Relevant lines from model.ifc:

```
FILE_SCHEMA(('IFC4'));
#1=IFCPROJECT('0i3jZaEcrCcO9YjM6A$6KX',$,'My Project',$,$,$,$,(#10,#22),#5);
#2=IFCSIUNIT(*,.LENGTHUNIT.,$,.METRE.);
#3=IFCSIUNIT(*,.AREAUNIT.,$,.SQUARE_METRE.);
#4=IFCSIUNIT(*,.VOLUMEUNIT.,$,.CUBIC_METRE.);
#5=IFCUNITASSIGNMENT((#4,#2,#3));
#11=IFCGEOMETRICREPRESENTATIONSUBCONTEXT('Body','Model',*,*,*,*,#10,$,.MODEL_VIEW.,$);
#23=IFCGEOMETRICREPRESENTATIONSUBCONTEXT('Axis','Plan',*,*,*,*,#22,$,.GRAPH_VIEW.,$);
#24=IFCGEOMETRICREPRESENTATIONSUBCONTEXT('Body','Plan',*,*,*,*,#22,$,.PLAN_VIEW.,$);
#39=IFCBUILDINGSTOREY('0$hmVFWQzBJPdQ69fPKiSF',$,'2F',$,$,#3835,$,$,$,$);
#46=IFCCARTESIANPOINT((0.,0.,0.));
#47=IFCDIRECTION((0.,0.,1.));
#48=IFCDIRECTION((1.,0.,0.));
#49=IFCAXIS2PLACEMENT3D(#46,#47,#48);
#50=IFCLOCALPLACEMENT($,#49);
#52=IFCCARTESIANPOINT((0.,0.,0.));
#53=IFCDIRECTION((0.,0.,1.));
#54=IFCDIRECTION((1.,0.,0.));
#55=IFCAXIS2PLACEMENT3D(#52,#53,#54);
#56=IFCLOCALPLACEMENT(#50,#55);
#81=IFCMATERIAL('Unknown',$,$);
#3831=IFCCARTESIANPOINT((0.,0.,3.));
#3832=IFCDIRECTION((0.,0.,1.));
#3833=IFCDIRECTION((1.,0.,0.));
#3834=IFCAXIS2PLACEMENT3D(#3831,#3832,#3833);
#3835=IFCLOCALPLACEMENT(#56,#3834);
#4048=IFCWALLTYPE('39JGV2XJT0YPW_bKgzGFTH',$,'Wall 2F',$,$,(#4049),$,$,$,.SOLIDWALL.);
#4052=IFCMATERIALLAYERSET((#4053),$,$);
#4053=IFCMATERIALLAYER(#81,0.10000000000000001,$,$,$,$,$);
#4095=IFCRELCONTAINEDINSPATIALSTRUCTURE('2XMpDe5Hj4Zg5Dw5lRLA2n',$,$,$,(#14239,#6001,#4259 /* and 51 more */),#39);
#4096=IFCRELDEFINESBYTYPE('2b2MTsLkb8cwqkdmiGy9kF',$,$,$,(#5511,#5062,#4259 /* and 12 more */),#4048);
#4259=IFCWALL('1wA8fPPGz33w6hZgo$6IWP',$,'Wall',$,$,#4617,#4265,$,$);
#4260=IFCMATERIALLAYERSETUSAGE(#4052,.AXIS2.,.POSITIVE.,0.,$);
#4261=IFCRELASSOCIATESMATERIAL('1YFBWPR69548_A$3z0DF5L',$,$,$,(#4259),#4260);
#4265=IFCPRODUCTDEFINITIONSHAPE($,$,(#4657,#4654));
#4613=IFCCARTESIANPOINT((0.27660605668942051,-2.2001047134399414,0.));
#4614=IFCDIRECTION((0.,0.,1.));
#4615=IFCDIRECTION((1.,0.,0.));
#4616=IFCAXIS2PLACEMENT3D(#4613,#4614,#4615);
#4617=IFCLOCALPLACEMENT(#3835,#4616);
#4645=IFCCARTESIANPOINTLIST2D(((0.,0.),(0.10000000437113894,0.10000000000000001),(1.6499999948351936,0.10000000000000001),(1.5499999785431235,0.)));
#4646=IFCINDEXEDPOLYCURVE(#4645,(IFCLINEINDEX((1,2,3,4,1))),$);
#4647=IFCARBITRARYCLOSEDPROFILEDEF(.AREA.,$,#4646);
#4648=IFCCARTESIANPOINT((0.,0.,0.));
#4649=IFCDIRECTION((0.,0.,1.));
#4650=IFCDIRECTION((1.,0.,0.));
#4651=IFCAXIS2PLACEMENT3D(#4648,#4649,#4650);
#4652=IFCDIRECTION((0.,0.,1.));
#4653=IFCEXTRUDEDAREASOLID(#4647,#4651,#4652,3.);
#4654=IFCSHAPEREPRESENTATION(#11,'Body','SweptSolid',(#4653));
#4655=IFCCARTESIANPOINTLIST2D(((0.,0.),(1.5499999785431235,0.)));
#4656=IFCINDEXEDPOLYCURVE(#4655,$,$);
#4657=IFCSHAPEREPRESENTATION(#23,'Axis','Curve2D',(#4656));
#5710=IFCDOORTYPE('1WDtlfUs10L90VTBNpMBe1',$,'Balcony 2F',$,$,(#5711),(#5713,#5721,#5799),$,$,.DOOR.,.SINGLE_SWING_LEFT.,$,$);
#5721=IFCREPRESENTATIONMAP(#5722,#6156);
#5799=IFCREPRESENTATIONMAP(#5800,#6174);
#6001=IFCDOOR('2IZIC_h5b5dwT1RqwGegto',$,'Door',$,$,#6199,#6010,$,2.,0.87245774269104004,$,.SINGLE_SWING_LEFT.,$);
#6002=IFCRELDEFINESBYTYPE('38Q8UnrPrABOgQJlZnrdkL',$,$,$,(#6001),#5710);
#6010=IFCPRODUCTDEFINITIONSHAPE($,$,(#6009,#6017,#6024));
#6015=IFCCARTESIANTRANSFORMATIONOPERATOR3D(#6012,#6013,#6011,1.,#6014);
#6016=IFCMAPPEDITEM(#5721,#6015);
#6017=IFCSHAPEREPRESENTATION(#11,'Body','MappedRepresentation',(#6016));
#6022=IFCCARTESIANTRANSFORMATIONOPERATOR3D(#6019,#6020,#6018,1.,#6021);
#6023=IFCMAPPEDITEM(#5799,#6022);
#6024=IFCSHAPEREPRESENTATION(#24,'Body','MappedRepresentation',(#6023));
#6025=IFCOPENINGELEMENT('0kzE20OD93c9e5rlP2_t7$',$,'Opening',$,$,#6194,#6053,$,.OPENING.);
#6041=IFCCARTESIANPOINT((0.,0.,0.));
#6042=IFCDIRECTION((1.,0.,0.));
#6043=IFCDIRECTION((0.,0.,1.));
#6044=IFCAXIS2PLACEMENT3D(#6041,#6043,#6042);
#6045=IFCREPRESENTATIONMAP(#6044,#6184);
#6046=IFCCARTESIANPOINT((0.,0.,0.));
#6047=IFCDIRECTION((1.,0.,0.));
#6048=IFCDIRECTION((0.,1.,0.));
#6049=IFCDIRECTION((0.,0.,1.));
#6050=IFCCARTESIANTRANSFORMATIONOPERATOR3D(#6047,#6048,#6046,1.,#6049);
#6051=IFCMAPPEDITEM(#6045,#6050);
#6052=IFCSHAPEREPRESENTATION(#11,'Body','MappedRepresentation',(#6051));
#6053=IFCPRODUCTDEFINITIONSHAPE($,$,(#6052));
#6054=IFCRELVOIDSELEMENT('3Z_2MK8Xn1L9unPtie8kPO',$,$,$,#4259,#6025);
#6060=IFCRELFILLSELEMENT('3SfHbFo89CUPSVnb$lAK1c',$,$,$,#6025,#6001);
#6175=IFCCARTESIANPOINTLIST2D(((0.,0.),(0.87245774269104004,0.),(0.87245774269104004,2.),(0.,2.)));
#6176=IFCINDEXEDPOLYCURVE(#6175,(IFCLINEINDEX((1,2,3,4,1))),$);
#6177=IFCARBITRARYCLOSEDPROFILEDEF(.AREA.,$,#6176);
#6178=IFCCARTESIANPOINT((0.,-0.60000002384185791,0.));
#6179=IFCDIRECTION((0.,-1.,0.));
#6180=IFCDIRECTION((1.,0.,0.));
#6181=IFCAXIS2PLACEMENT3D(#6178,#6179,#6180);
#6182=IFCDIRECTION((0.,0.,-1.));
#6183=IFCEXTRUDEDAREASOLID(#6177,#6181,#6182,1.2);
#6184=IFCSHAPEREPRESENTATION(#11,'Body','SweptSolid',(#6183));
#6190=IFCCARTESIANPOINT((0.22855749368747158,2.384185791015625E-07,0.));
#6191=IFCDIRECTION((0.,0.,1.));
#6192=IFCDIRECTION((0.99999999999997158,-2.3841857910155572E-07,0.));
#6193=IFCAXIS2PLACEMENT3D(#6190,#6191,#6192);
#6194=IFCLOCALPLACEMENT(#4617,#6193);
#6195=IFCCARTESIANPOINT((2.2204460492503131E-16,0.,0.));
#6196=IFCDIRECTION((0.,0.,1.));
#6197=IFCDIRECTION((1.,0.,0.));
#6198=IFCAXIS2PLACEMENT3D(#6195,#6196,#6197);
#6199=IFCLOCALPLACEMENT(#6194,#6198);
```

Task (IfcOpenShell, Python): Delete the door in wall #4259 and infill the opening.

```python
import ifcopenshell
import ifcopenshell.api.feature
import ifcopenshell.api.root
import ifcopenshell.geom
import ifcopenshell.util.shape

model = ifcopenshell.open("model.ifc")
settings = ifcopenshell.geom.settings()


def volume(element):
    """Net volume in cubic metres, openings subtracted."""
    shape = ifcopenshell.geom.create_shape(settings, element)
    return ifcopenshell.util.shape.get_volume(shape.geometry)


door = model.by_guid("2IZIC_h5b5dwT1RqwGegto")
opening = door.FillsVoids[0].RelatingOpeningElement
wall = opening.VoidsElements[0].RelatingBuildingElement
before = volume(wall)

ifcopenshell.api.root.remove_product(model, product=door)
ifcopenshell.api.feature.remove_feature(model, feature=opening)

after = volume(wall)

print(f"wall volume {before:.3f} -> {after:.3f} m3")

model.write("model_updated.ifc")
```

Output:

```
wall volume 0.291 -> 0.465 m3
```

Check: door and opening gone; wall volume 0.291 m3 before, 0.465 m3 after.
